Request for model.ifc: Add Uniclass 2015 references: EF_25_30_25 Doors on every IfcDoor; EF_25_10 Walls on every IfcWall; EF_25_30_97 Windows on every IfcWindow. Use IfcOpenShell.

First a look at what the model holds.

```python
import ifcopenshell

model = ifcopenshell.open("model.ifc")
print(model.schema)
print("classifications:", [c.Name for c in model.by_type("IfcClassification")])
for ifc_class in ("IfcDoor", "IfcRoof", "IfcStair", "IfcWall", "IfcWindow"):
    print(ifc_class, len(model.by_type(ifc_class)))
```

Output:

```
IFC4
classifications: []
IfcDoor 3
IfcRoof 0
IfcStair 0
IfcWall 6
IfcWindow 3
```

```python
import ifcopenshell
import ifcopenshell.api.classification

model = ifcopenshell.open("model.ifc")

system = ifcopenshell.api.classification.add_classification(model, classification="Uniclass 2015")

codes = {
    "IfcDoor": ("EF_25_30_25", "Doors"),
    "IfcWall": ("EF_25_10", "Walls"),
    "IfcWindow": ("EF_25_30_97", "Windows"),
}
for ifc_class, (code, name) in codes.items():
    products = model.by_type(ifc_class)
    ifcopenshell.api.classification.add_reference(
        model, products=products, classification=system, identification=code, name=name
    )
    print(code, len(products))

model.write("model_edited.ifc")
```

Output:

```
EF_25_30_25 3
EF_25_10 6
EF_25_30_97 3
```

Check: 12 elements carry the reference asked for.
